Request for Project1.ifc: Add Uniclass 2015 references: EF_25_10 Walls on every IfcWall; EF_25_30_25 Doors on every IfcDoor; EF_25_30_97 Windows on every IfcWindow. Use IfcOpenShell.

First a look at what the model holds.

```python
import ifcopenshell

model = ifcopenshell.open("Project1.ifc")
print(model.schema)
print("classifications:", [c.Name for c in model.by_type("IfcClassification")])
for ifc_class in ("IfcDoor", "IfcRoof", "IfcStair", "IfcWall", "IfcWindow"):
    print(ifc_class, len(model.by_type(ifc_class)))
```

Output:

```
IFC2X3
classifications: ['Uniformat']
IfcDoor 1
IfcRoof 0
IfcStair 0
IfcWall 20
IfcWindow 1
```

```python
import ifcopenshell
import ifcopenshell.api.classification

model = ifcopenshell.open("Project1.ifc")

# IFC2X3 requires Source and Edition and has no link from the project to the system.
system = model.create_entity("IfcClassification", Source="NBS", Edition="2015", Name="Uniclass 2015")

codes = {
    "IfcWall": ("EF_25_10", "Walls"),
    "IfcDoor": ("EF_25_30_25", "Doors"),
    "IfcWindow": ("EF_25_30_97", "Windows"),
}
for ifc_class, (code, name) in codes.items():
    products = model.by_type(ifc_class)
    ifcopenshell.api.classification.add_reference(
        model, products=products, classification=system, identification=code, name=name
    )
    print(code, len(products))

model.write("Project1_updated.ifc")
```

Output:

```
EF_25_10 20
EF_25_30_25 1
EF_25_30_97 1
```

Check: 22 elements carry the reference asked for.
